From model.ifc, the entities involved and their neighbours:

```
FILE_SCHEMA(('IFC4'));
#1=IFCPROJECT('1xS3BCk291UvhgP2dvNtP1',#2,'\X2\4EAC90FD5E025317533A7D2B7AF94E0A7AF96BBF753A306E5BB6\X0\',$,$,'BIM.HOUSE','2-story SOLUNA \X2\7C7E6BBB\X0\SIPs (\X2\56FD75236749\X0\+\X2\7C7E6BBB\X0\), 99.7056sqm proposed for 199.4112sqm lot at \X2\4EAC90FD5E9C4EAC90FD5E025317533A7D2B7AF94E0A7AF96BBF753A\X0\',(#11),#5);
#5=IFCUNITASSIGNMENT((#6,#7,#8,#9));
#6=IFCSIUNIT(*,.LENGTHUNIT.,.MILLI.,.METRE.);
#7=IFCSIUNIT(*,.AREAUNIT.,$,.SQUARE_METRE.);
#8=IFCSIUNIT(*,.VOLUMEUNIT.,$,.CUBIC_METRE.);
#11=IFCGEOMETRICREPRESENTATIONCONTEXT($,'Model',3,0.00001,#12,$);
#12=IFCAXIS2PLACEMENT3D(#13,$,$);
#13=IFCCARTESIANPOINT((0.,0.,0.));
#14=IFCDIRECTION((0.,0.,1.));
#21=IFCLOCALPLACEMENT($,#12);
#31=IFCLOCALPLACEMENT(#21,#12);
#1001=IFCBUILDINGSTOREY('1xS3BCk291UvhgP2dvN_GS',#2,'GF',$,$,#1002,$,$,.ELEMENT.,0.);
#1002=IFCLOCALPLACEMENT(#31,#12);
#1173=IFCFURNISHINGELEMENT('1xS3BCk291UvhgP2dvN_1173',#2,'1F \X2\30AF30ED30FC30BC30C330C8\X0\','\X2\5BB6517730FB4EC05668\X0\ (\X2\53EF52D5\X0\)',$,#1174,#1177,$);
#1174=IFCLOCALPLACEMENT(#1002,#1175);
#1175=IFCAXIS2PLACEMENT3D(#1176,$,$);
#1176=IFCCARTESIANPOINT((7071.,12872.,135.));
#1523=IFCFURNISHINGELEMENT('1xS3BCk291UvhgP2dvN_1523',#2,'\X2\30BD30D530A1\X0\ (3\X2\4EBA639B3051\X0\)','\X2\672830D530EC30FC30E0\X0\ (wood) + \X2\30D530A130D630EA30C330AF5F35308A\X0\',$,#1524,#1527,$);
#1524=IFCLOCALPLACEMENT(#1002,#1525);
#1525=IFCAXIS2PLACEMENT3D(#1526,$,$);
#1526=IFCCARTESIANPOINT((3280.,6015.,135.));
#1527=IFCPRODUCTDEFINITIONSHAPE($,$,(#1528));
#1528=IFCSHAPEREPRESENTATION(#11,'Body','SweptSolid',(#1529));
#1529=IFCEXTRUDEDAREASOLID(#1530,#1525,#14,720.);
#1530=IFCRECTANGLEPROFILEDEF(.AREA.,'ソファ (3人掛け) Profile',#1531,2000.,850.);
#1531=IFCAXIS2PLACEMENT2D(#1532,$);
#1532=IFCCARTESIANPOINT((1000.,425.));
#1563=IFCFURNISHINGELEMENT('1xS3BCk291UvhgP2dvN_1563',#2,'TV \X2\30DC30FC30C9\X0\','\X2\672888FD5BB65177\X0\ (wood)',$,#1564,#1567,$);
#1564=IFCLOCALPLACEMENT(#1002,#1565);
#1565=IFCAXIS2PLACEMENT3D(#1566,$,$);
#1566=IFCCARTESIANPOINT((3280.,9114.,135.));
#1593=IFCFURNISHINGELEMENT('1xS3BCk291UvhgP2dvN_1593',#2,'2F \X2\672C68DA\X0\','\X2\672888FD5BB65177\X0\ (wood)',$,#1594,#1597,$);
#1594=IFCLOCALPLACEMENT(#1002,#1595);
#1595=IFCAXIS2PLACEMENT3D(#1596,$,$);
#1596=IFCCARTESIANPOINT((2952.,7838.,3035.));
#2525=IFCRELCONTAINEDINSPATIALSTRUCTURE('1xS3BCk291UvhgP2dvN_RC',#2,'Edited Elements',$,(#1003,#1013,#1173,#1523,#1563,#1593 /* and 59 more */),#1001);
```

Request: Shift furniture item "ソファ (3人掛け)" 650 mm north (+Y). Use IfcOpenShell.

```python
import ifcopenshell
import ifcopenshell.api.geometry
import ifcopenshell.util.placement
import ifcopenshell.util.unit

model = ifcopenshell.open("model.ifc")
unit_scale = ifcopenshell.util.unit.calculate_unit_scale(model)

item = model.by_id(1523)
matrix = ifcopenshell.util.placement.get_local_placement(item.ObjectPlacement)
matrix[1, 3] += 0.65 / unit_scale
ifcopenshell.api.geometry.edit_object_placement(model, product=item, matrix=matrix, is_si=False)

print(ifcopenshell.util.placement.get_local_placement(item.ObjectPlacement).round(3) + 0.0)

model.write("model_v2.ifc")
```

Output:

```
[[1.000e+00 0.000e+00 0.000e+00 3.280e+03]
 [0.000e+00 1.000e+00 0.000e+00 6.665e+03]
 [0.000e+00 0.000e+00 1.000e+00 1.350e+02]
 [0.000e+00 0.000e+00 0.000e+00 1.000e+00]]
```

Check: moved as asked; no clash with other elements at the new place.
